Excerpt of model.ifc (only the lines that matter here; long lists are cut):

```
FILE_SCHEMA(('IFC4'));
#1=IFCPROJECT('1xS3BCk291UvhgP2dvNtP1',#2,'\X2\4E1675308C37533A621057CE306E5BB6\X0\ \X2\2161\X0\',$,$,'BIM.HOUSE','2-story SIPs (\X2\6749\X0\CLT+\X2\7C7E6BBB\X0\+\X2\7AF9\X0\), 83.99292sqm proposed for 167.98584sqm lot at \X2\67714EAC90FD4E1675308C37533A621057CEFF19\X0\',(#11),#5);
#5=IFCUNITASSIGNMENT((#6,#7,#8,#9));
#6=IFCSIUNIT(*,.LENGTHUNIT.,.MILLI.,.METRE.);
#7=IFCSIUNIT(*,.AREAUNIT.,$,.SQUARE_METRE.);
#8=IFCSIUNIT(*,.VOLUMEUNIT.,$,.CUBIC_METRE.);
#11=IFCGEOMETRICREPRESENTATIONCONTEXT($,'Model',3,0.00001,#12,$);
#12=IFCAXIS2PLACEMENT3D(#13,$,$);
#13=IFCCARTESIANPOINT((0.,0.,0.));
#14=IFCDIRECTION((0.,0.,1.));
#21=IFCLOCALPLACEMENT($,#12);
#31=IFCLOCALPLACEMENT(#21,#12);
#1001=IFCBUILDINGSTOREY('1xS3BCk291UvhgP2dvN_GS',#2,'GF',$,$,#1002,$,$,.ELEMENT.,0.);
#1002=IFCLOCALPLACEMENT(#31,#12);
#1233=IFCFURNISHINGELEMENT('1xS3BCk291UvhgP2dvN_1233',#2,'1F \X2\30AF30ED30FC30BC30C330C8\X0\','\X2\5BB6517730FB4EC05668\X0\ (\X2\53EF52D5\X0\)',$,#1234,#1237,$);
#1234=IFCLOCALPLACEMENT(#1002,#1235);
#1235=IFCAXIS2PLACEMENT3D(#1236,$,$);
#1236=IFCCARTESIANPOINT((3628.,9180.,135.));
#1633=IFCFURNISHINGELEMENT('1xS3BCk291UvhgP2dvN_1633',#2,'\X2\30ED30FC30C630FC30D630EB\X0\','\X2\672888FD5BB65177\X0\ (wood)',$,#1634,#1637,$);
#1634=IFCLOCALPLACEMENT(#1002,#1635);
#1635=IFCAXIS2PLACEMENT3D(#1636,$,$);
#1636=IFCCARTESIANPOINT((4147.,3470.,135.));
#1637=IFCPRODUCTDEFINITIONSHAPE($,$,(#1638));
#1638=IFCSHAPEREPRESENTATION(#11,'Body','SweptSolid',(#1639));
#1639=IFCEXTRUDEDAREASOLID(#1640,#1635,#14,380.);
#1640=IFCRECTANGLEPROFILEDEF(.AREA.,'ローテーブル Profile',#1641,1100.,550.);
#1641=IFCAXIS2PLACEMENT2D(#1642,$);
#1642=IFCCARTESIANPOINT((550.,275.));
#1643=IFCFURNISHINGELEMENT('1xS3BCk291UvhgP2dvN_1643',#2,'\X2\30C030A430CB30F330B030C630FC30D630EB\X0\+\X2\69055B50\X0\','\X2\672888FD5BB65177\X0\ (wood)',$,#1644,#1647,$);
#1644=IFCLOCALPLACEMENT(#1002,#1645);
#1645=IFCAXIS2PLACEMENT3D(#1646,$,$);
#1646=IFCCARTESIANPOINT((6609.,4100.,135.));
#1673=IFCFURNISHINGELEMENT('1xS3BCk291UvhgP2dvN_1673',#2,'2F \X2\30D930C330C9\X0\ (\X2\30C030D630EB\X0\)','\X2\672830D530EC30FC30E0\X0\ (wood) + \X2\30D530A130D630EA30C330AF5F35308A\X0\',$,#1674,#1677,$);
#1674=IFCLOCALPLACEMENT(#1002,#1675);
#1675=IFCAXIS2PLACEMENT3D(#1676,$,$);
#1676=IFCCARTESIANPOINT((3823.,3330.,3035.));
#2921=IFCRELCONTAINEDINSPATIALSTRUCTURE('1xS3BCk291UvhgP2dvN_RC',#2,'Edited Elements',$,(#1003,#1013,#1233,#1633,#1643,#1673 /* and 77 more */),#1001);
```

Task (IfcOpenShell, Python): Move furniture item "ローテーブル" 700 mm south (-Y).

```python
import ifcopenshell
import ifcopenshell.api.geometry
import ifcopenshell.util.placement
import ifcopenshell.util.unit

model = ifcopenshell.open("model.ifc")
unit_scale = ifcopenshell.util.unit.calculate_unit_scale(model)

item = model.by_guid("1xS3BCk291UvhgP2dvN_1633")
matrix = ifcopenshell.util.placement.get_local_placement(item.ObjectPlacement)
matrix[1, 3] -= 0.7 / unit_scale
ifcopenshell.api.geometry.edit_object_placement(model, product=item, matrix=matrix, is_si=False)

print(ifcopenshell.util.placement.get_local_placement(item.ObjectPlacement).round(3) + 0.0)

model.write("model_updated.ifc")
```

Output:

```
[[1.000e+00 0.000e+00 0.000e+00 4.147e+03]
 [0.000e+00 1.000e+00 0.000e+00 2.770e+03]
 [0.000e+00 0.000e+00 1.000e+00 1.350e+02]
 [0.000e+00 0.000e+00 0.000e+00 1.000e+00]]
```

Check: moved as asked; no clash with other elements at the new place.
